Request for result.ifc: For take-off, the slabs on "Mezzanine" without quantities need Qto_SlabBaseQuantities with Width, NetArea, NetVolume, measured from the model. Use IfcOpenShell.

First a look at what the model holds.

```python
import ifcopenshell
import ifcopenshell.util.element
import ifcopenshell.util.unit

model = ifcopenshell.open("result.ifc")
print(model.schema)
for unit_type in ("LENGTHUNIT", "AREAUNIT", "VOLUMEUNIT"):
    print(unit_type, ifcopenshell.util.unit.calculate_unit_scale(model, unit_type))
storey = next(s for s in model.by_type("IfcBuildingStorey") if s.Name == "Mezzanine")
slabs = [e for e in ifcopenshell.util.element.get_decomposition(storey) if e.is_a("IfcSlab")]
for e in sorted(slabs, key=lambda e: e.id()):
    print(e.id(), e.is_a(), e.Name, list(ifcopenshell.util.element.get_psets(e, qtos_only=True)), sep=" | ")
```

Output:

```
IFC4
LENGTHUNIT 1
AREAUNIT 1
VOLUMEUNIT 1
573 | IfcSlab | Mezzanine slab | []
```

```python
import ifcopenshell
import ifcopenshell.api.pset
import ifcopenshell.geom
import ifcopenshell.util.element
import ifcopenshell.util.shape
import ifcopenshell.util.unit

model = ifcopenshell.open("result.ifc")
unit_scale = ifcopenshell.util.unit.calculate_unit_scale(model)
area_scale = ifcopenshell.util.unit.calculate_unit_scale(model, "AREAUNIT")
volume_scale = ifcopenshell.util.unit.calculate_unit_scale(model, "VOLUMEUNIT")
settings = ifcopenshell.geom.settings()

storey = next(s for s in model.by_type("IfcBuildingStorey") if s.Name == "Mezzanine")
slabs = [e for e in ifcopenshell.util.element.get_decomposition(storey) if e.is_a("IfcSlab")]

for e in sorted(slabs, key=lambda e: e.id()):
    if ifcopenshell.util.element.get_psets(e, qtos_only=True, should_inherit=False):
        continue
    # Geometry comes back in metres, in the element's own axes.
    shape = ifcopenshell.geom.create_shape(settings, e)
    values = {
        "Width": ifcopenshell.util.shape.get_z(shape.geometry) / unit_scale,
        "NetArea": ifcopenshell.util.shape.get_footprint_area(shape.geometry) / area_scale,
        "NetVolume": ifcopenshell.util.shape.get_volume(shape.geometry) / volume_scale,
    }
    qto = ifcopenshell.api.pset.add_qto(model, product=e, name="Qto_SlabBaseQuantities")
    ifcopenshell.api.pset.edit_qto(model, qto=qto, properties=values)
    print(e.id(), {k: round(v, 3) for k, v in values.items()})

model.write("result-out.ifc")
```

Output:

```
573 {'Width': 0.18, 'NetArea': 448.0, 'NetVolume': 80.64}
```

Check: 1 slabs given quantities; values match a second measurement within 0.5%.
